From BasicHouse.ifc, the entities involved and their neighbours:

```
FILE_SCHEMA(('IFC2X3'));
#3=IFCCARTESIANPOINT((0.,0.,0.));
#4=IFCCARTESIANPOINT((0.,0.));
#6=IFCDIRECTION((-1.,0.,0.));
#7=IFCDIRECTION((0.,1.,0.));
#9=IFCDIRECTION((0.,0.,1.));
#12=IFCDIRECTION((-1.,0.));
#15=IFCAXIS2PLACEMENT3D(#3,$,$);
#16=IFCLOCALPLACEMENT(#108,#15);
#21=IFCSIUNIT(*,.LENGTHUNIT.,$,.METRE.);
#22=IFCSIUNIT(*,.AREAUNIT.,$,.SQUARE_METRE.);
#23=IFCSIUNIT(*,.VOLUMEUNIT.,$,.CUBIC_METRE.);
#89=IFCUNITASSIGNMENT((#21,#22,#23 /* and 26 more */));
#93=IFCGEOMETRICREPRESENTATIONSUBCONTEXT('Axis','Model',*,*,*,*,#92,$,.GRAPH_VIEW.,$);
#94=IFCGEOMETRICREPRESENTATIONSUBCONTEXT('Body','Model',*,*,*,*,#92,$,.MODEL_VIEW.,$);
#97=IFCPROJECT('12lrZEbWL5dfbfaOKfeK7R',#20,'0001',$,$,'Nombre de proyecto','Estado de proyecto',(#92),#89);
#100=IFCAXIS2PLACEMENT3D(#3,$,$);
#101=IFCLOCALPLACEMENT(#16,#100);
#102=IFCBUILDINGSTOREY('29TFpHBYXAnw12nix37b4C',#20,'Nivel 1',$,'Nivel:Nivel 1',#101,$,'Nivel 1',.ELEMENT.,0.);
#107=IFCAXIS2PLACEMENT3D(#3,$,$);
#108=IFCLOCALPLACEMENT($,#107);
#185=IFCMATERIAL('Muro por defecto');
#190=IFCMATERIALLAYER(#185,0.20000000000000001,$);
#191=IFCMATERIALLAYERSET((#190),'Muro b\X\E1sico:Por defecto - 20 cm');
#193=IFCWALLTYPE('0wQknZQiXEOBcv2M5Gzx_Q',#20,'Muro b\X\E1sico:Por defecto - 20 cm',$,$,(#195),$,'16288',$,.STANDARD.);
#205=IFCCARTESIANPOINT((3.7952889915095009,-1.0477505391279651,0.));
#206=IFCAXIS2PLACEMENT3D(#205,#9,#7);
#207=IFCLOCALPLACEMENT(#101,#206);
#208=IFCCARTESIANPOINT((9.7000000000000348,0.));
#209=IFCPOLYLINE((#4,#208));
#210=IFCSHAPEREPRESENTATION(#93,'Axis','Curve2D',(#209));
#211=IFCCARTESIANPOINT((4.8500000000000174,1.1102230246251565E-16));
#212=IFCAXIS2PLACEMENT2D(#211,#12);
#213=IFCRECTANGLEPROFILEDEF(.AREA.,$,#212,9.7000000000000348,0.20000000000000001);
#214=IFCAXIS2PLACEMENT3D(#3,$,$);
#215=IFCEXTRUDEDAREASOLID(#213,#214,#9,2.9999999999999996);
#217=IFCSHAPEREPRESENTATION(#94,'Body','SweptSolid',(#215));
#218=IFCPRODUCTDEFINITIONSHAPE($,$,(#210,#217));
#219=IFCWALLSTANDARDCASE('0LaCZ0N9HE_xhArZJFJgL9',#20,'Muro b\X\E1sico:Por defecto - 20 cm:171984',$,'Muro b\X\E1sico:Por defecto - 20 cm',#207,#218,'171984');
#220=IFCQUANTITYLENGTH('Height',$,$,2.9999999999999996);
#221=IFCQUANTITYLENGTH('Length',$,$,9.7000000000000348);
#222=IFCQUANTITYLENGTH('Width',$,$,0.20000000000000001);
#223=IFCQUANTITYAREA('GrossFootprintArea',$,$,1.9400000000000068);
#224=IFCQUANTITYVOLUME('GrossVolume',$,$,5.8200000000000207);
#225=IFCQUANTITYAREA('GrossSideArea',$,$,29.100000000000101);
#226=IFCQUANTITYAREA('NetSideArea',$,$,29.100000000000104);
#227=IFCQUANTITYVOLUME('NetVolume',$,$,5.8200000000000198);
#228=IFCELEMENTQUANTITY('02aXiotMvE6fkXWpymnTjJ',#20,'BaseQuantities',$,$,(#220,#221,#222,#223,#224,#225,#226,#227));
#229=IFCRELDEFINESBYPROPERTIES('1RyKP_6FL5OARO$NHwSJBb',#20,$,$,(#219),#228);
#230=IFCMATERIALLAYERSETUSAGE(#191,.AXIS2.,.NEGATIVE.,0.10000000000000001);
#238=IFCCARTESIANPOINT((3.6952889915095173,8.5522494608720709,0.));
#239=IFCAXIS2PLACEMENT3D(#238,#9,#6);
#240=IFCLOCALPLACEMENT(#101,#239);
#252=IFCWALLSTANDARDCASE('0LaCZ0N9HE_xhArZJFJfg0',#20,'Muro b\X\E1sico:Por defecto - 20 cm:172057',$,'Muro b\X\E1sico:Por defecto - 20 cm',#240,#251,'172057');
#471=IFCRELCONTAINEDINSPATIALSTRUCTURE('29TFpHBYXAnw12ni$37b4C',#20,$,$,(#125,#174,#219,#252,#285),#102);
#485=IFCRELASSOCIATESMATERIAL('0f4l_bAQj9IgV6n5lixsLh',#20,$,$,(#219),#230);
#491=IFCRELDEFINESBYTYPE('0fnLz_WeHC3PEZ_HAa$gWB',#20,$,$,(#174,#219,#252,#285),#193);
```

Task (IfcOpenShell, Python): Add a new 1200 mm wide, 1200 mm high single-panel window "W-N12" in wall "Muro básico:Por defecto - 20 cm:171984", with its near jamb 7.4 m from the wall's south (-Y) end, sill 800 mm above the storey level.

```python
import numpy as np
import ifcopenshell
import ifcopenshell.api.feature
import ifcopenshell.api.geometry
import ifcopenshell.api.pset
import ifcopenshell.api.root
import ifcopenshell.api.spatial
import ifcopenshell.api.type
import ifcopenshell.geom
import ifcopenshell.util.element
import ifcopenshell.util.placement
import ifcopenshell.util.representation
import ifcopenshell.util.shape
import ifcopenshell.util.unit

model = ifcopenshell.open("BasicHouse.ifc")
unit_scale = ifcopenshell.util.unit.calculate_unit_scale(model)
area_scale = ifcopenshell.util.unit.calculate_unit_scale(model, "AREAUNIT")
volume_scale = ifcopenshell.util.unit.calculate_unit_scale(model, "VOLUMEUNIT")
settings = ifcopenshell.geom.settings()


def volume(element):
    """Net volume in cubic metres, openings subtracted."""
    shape = ifcopenshell.geom.create_shape(settings, element)
    return ifcopenshell.util.shape.get_volume(shape.geometry)


wall = model.by_guid("0LaCZ0N9HE_xhArZJFJgL9")
storey = ifcopenshell.util.element.get_container(wall, ifc_class="IfcBuildingStorey")
context = ifcopenshell.util.representation.get_context(model, "Model", "Body", "MODEL_VIEW")
before = volume(wall)

width, height, from_end, sill = 1.2, 1.2, 7.4, 0.8  # metres

# The wall runs along its own X axis, and the end named is its -X end.
wall_shape = ifcopenshell.geom.create_shape(settings, wall)
x, y, z = ifcopenshell.util.shape.get_vertices(wall_shape.geometry).T
start = x.min() + from_end
face, thickness = float(y.min()), float(y.max() - y.min())
wall_matrix = ifcopenshell.util.placement.get_local_placement(wall.ObjectPlacement)
level = ifcopenshell.util.placement.get_local_placement(storey.ObjectPlacement)[2, 3]


def in_wall(x, y):
    """Placement at x, y metres in the wall's axes, at sill height."""
    matrix = wall_matrix.copy()
    matrix[:, 3] = wall_matrix @ np.array([x / unit_scale, y / unit_scale, 0.0, 1.0])
    matrix[2, 3] = level + sill / unit_scale
    return matrix


# Opening: a box that overshoots both wall faces by 50 mm.
opening = ifcopenshell.api.root.create_entity(model, ifc_class="IfcOpeningElement")
box = ifcopenshell.api.geometry.add_wall_representation(
    model, context=context, length=width, height=height, thickness=thickness + 0.1
)
ifcopenshell.api.geometry.assign_representation(model, product=opening, representation=box)
ifcopenshell.api.geometry.edit_object_placement(model, product=opening, matrix=in_wall(start, face - 0.05), is_si=False)
ifcopenshell.api.feature.add_feature(model, feature=opening, element=wall)

window = ifcopenshell.api.root.create_entity(model, ifc_class="IfcWindow", name="W-N12")
window.OverallWidth, window.OverallHeight = width / unit_scale, height / unit_scale
body = ifcopenshell.api.geometry.add_window_representation(
    model,
    context=context,
    overall_width=window.OverallWidth,
    overall_height=window.OverallHeight,
    partition_type="SINGLE_PANEL",
)
ifcopenshell.api.geometry.assign_representation(model, product=window, representation=body)
ifcopenshell.api.spatial.assign_container(model, products=[window], relating_structure=storey)
fills = ifcopenshell.api.feature.add_filling(model, opening=opening, element=window)
fills.OwnerHistory = window.OwnerHistory  # required in IFC2X3

# IFC2X3 keeps the operation on the window style.
style = ifcopenshell.api.root.create_entity(model, ifc_class="IfcWindowStyle", name="W-N12")
style.OperationType, style.ConstructionType = "SINGLE_PANEL", "NOTDEFINED"
style.ParameterTakesPrecedence = style.Sizeable = False
ifcopenshell.api.type.assign_type(model, related_objects=[window], relating_type=style)

# Centre the window in the wall's thickness.
ifcopenshell.api.geometry.edit_object_placement(model, product=window, matrix=in_wall(start, face), is_si=False)
window_shape = ifcopenshell.geom.create_shape(settings, window)
depth = ifcopenshell.util.shape.get_vertices(window_shape.geometry)[:, 1]
offset = face + thickness / 2 - (depth.min() + depth.max()) / 2
ifcopenshell.api.geometry.edit_object_placement(model, product=window, matrix=in_wall(start, offset), is_si=False)

after = volume(wall)

# Update the wall's stored quantities.
qto = model.by_id(ifcopenshell.util.element.get_pset(wall, "BaseQuantities", should_inherit=False)["id"])
ifcopenshell.api.pset.edit_qto(model, qto=qto, properties={
    "NetSideArea": after / thickness / area_scale,
    "NetVolume": after / volume_scale,
})

print(f"wall volume {before:.3f} -> {after:.3f} m3")

model.write("BasicHouse_updated.ifc")
```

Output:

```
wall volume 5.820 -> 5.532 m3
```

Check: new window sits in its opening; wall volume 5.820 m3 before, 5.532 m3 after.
